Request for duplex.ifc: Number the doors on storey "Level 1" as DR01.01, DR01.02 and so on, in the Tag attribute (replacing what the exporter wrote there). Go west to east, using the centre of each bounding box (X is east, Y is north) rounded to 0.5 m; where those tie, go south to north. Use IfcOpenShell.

First a look at what the model holds.

```python
import ifcopenshell
import ifcopenshell.util.element
import ifcopenshell.util.placement

model = ifcopenshell.open("duplex.ifc")
print(model.schema)
storey = next(s for s in model.by_type("IfcBuildingStorey") if s.Name == "Level 1")
doors = [e for e in ifcopenshell.util.element.get_decomposition(storey) if e.is_a("IfcDoor")]
for e in sorted(doors, key=lambda e: e.id()):
    origin = ifcopenshell.util.placement.get_local_placement(e.ObjectPlacement)[:3, 3]
    print(e.id(), e.Tag, e.Name, origin.round(2) + 0.0, sep=" | ")
```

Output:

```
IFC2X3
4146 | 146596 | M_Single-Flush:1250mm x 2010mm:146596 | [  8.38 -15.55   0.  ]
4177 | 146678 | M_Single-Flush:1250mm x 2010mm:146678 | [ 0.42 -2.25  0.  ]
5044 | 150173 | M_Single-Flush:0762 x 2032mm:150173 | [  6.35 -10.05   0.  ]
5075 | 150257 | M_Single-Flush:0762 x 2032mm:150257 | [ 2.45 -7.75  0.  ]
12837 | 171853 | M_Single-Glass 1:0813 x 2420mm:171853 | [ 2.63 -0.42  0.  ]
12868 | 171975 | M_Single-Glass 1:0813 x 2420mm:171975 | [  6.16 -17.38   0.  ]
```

```python
import ifcopenshell
import ifcopenshell.geom
import ifcopenshell.util.element
import ifcopenshell.util.shape

model = ifcopenshell.open("duplex.ifc")
settings = ifcopenshell.geom.settings()
settings.set("use-world-coords", True)


def centre(element):
    shape = ifcopenshell.geom.create_shape(settings, element)
    return ifcopenshell.util.shape.get_bbox_centroid(shape.geometry)


storey = next(s for s in model.by_type("IfcBuildingStorey") if s.Name == "Level 1")
doors = [e for e in ifcopenshell.util.element.get_decomposition(storey) if e.is_a("IfcDoor")]

# Insertion points can sit at a corner or the storey origin, so sort by the geometry (in metres).
centres = {e: centre(e) for e in doors}
doors.sort(key=lambda e: (round(centres[e][0] / 0.5), centres[e][1]))

for i, e in enumerate(doors, start=1):
    number = f"DR01.{i:02d}"
    e.Tag = number
    print(e.id(), number)

model.write("duplex_edited.ifc")
```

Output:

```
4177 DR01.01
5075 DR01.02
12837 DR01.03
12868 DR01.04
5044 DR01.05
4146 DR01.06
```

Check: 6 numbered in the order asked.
